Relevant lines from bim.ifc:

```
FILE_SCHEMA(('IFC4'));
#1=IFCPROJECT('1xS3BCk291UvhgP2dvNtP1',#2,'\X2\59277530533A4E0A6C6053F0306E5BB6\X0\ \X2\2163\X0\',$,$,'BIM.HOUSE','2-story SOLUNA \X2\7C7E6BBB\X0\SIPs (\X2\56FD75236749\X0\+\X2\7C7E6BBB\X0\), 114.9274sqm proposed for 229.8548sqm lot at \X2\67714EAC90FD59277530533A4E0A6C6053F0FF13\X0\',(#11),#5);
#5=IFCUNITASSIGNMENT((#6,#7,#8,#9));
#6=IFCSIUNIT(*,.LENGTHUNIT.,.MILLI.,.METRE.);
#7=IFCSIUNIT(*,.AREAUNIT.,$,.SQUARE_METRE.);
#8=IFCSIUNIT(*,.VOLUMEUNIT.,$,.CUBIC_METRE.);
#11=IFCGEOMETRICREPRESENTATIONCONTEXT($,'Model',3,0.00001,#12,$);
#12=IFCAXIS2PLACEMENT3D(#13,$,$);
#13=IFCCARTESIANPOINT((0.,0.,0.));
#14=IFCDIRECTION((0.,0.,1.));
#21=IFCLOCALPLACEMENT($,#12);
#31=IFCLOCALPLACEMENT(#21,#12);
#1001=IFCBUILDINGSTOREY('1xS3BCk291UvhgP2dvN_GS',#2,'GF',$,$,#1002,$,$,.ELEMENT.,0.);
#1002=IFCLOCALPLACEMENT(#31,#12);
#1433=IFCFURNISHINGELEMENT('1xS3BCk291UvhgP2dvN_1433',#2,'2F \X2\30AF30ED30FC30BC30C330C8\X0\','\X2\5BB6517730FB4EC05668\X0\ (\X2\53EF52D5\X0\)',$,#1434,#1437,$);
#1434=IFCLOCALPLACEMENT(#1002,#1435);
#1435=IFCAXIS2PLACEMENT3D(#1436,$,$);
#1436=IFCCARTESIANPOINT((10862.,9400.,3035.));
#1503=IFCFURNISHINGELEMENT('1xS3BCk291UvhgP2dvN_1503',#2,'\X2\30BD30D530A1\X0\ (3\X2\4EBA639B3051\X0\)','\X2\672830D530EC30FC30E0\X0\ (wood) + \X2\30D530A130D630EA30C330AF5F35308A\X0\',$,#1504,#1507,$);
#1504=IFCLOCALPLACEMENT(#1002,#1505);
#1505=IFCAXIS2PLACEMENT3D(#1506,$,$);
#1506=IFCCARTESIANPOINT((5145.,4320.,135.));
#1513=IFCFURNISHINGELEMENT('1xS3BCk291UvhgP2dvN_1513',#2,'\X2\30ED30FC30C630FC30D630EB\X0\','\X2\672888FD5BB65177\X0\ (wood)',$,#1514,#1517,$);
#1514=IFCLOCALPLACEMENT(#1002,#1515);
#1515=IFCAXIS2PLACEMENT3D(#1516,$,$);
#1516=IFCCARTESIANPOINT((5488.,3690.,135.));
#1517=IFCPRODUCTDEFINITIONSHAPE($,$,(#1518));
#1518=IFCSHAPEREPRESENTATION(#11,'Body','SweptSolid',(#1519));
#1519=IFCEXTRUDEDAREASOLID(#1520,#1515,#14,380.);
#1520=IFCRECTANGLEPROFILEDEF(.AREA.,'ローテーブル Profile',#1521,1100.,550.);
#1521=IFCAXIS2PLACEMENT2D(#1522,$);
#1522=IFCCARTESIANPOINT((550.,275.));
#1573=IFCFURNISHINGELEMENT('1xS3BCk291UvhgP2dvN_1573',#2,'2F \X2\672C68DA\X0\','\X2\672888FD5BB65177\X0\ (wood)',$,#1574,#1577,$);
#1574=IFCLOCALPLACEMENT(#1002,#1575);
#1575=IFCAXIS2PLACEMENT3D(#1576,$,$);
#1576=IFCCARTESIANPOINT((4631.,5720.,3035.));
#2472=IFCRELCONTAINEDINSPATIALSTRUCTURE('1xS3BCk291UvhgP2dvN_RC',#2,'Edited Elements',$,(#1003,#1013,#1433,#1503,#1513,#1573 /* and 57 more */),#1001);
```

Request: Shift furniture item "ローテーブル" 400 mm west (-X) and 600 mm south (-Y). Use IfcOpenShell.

```python
import ifcopenshell
import ifcopenshell.api.geometry
import ifcopenshell.util.placement
import ifcopenshell.util.unit

model = ifcopenshell.open("bim.ifc")
unit_scale = ifcopenshell.util.unit.calculate_unit_scale(model)

item = model.by_guid("1xS3BCk291UvhgP2dvN_1513")
matrix = ifcopenshell.util.placement.get_local_placement(item.ObjectPlacement)
matrix[0, 3] -= 0.4 / unit_scale
matrix[1, 3] -= 0.6 / unit_scale
ifcopenshell.api.geometry.edit_object_placement(model, product=item, matrix=matrix, is_si=False)

print(ifcopenshell.util.placement.get_local_placement(item.ObjectPlacement).round(3) + 0.0)

model.write("bim_rev.ifc")
```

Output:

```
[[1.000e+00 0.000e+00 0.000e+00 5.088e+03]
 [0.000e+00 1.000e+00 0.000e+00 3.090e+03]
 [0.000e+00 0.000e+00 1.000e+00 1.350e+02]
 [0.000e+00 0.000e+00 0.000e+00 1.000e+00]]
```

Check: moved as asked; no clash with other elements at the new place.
